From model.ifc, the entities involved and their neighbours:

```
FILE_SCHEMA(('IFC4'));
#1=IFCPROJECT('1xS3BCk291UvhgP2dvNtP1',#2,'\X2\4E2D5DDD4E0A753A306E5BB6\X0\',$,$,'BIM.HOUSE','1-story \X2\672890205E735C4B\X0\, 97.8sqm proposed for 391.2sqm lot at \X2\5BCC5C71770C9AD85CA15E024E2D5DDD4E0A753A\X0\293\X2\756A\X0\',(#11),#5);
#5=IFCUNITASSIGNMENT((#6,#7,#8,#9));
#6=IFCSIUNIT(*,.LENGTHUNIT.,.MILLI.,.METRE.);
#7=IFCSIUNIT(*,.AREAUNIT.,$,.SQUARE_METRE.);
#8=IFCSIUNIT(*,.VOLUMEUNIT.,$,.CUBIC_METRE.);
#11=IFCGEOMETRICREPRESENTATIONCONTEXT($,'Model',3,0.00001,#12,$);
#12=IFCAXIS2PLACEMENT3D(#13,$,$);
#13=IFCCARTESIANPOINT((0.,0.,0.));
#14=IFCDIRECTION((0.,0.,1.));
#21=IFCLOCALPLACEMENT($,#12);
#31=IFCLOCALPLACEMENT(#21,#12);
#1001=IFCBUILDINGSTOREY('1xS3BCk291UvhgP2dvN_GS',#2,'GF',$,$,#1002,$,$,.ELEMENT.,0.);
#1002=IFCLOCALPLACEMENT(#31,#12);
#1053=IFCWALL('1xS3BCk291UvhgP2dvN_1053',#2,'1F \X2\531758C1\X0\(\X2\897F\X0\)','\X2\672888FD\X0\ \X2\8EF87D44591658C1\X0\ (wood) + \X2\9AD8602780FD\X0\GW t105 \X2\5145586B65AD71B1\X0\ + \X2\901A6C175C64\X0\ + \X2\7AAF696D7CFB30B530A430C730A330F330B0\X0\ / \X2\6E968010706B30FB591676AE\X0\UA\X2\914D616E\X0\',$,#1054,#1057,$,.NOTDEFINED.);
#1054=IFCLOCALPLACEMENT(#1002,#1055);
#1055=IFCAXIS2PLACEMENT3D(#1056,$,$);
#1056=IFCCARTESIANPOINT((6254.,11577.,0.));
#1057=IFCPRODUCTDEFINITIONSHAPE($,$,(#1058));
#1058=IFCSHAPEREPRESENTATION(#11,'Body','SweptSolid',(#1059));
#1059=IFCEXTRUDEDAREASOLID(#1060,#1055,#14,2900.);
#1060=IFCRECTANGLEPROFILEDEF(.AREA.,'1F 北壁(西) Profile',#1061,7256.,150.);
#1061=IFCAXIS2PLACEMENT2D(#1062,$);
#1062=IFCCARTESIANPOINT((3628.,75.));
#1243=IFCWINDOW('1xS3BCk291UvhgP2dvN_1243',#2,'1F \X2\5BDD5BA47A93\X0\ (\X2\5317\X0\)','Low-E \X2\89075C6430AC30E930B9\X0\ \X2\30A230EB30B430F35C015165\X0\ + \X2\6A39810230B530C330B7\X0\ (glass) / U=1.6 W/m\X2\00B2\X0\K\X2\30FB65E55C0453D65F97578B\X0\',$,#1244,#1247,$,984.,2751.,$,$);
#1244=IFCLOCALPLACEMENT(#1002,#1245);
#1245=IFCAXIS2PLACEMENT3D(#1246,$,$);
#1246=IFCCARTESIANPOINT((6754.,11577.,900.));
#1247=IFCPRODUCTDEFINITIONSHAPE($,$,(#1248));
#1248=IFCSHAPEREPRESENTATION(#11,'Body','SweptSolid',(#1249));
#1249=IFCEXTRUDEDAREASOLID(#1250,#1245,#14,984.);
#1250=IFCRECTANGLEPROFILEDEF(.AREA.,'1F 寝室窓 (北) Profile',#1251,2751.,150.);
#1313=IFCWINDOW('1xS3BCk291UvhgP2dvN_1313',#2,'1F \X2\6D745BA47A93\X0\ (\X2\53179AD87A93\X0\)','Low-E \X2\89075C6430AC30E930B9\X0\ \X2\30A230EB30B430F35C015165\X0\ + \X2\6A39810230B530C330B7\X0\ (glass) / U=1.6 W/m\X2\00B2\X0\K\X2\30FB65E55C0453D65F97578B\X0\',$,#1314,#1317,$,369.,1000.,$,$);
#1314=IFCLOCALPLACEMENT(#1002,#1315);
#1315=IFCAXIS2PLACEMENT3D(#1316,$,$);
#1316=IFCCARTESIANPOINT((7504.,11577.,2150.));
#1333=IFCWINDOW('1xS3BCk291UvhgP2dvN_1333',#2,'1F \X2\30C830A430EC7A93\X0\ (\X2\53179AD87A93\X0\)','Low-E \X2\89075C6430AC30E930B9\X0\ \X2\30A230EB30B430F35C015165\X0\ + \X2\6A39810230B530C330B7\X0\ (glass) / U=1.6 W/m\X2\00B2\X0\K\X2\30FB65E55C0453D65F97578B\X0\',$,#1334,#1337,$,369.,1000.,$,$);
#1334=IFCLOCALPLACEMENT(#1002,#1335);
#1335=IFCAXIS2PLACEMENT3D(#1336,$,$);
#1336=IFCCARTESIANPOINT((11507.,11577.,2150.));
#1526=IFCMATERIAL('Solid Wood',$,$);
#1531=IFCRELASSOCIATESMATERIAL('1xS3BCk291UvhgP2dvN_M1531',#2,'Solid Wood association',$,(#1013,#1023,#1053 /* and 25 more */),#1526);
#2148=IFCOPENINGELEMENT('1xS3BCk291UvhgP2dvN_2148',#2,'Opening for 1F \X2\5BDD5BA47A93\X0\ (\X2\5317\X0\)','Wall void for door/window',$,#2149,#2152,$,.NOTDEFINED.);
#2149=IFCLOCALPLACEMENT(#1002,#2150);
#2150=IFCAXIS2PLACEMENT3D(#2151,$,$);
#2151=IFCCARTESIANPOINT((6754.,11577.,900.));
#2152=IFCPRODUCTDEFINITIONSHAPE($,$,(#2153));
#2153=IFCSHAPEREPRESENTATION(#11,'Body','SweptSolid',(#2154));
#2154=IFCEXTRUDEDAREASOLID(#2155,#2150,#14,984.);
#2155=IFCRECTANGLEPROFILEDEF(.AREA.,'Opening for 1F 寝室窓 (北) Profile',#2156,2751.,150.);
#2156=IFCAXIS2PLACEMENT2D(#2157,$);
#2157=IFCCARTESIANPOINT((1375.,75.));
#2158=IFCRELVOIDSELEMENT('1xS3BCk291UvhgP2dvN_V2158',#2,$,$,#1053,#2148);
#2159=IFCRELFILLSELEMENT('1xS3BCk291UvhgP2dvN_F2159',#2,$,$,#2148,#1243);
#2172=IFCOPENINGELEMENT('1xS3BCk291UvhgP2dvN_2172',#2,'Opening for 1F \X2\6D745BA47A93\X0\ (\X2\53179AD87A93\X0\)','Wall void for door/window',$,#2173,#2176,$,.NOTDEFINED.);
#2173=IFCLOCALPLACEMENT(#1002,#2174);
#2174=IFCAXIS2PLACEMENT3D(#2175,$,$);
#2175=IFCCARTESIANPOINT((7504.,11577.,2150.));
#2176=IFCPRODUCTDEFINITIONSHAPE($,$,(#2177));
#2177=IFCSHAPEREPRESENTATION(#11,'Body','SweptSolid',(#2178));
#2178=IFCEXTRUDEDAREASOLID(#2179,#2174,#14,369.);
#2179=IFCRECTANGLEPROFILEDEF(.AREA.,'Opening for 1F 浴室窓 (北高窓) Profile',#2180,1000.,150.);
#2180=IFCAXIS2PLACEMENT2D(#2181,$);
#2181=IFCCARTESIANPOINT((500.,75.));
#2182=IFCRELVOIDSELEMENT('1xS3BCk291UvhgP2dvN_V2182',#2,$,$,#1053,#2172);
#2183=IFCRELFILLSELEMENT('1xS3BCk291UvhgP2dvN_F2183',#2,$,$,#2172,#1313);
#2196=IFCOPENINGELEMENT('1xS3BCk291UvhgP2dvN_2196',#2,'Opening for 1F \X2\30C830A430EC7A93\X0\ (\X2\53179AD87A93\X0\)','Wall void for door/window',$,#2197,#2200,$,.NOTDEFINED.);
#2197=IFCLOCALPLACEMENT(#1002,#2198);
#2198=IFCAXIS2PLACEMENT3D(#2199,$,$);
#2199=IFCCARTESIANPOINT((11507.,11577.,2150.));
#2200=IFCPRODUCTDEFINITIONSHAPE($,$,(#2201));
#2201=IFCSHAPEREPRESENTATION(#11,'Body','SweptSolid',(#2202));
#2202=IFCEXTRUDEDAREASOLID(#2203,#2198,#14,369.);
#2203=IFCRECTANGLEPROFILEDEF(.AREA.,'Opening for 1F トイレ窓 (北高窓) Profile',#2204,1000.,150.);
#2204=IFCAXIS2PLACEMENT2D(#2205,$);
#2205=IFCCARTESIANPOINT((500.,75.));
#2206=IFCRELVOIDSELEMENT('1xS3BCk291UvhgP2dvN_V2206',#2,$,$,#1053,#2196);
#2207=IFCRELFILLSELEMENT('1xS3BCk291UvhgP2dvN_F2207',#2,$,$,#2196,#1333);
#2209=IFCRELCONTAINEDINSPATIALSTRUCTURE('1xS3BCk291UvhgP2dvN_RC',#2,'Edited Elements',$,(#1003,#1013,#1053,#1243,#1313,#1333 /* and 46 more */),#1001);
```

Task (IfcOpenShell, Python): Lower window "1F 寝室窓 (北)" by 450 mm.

```python
import numpy as np
import ifcopenshell
import ifcopenshell.api.geometry
import ifcopenshell.util.placement
import ifcopenshell.util.unit

model = ifcopenshell.open("model.ifc")
unit_scale = ifcopenshell.util.unit.calculate_unit_scale(model)

window = model.by_guid("1xS3BCk291UvhgP2dvN_1243")
opening = window.FillsVoids[0].RelatingOpeningElement
dz = -0.45 / unit_scale

shift = np.array([0.0, 0.0, dz])
# The window is not placed relative to its opening, so move both.
for product in (opening, window):
    matrix = ifcopenshell.util.placement.get_local_placement(product.ObjectPlacement)
    matrix[:3, 3] += shift
    ifcopenshell.api.geometry.edit_object_placement(model, product=product, matrix=matrix, is_si=False)

print(f"moved by {dz * unit_scale:+.3f} m")

model.write("model_edited.ifc")
```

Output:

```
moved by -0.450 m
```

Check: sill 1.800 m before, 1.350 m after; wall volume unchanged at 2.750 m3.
